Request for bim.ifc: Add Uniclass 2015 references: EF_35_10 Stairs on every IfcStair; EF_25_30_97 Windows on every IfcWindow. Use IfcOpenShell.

First a look at what the model holds.

```python
import ifcopenshell

model = ifcopenshell.open("bim.ifc")
print(model.schema)
print("classifications:", [c.Name for c in model.by_type("IfcClassification")])
for ifc_class in ("IfcDoor", "IfcRoof", "IfcStair", "IfcWall", "IfcWindow"):
    print(ifc_class, len(model.by_type(ifc_class)))
```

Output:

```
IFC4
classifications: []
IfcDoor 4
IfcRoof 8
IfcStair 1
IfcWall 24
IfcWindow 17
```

```python
import ifcopenshell
import ifcopenshell.api.classification

model = ifcopenshell.open("bim.ifc")

system = ifcopenshell.api.classification.add_classification(model, classification="Uniclass 2015")

codes = {
    "IfcStair": ("EF_35_10", "Stairs"),
    "IfcWindow": ("EF_25_30_97", "Windows"),
}
for ifc_class, (code, name) in codes.items():
    products = model.by_type(ifc_class)
    ifcopenshell.api.classification.add_reference(
        model, products=products, classification=system, identification=code, name=name
    )
    print(code, len(products))

model.write("bim_updated.ifc")
```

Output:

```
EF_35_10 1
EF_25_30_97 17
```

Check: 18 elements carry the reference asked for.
